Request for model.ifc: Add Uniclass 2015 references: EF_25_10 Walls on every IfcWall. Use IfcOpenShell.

First a look at what the model holds.

```python
import ifcopenshell

model = ifcopenshell.open("model.ifc")
print(model.schema)
print("classifications:", [c.Name for c in model.by_type("IfcClassification")])
for ifc_class in ("IfcDoor", "IfcRoof", "IfcStair", "IfcWall", "IfcWindow"):
    print(ifc_class, len(model.by_type(ifc_class)))
```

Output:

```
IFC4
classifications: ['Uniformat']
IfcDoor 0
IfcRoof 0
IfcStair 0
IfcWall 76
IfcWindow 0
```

```python
import ifcopenshell
import ifcopenshell.api.classification

model = ifcopenshell.open("model.ifc")

system = ifcopenshell.api.classification.add_classification(model, classification="Uniclass 2015")

codes = {
    "IfcWall": ("EF_25_10", "Walls"),
}
for ifc_class, (code, name) in codes.items():
    products = model.by_type(ifc_class)
    ifcopenshell.api.classification.add_reference(
        model, products=products, classification=system, identification=code, name=name
    )
    print(code, len(products))

model.write("model_v2.ifc")
```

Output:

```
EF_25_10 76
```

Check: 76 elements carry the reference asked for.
